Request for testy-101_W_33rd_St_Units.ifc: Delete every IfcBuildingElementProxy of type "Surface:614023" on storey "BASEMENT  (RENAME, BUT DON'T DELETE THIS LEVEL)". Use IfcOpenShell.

First a look at what the model holds.

```python
import ifcopenshell
import ifcopenshell.util.element

model = ifcopenshell.open("testy-101_W_33rd_St_Units.ifc")
print(model.schema)
storey = next(s for s in model.by_type("IfcBuildingStorey") if s.Name == "BASEMENT  (RENAME, BUT DON'T DELETE THIS LEVEL)")
proxies = [e for e in ifcopenshell.util.element.get_decomposition(storey) if e.is_a("IfcBuildingElementProxy")]
seen = {}
for e in proxies:
    element_type = ifcopenshell.util.element.get_type(e)
    name = element_type.Name if element_type not in (None, e) else None
    seen[name] = seen.get(name, 0) + 1
for name, count in sorted(seen.items(), key=str):
    print(count, "x", name)
```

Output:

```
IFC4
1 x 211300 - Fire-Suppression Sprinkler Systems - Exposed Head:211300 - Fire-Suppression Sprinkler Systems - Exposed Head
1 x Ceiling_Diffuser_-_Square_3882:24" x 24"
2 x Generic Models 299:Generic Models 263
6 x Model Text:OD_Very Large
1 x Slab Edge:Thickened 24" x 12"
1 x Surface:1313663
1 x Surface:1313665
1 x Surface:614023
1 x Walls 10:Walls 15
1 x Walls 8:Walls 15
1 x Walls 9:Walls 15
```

```python
import ifcopenshell
import ifcopenshell.api.root
import ifcopenshell.util.element

model = ifcopenshell.open("testy-101_W_33rd_St_Units.ifc")

storey = next(s for s in model.by_type("IfcBuildingStorey") if s.Name == "BASEMENT  (RENAME, BUT DON'T DELETE THIS LEVEL)")
proxies = [e for e in ifcopenshell.util.element.get_decomposition(storey) if e.is_a("IfcBuildingElementProxy")]
targets = [e for e in proxies if (t := ifcopenshell.util.element.get_type(e)) not in (None, e) and t.Name == "Surface:614023"]

for e in targets:
    ifcopenshell.api.root.remove_product(model, product=e)
print(len(targets), "removed")

model.write("testy-101_W_33rd_St_Units_updated.ifc")
```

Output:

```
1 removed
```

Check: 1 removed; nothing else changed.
